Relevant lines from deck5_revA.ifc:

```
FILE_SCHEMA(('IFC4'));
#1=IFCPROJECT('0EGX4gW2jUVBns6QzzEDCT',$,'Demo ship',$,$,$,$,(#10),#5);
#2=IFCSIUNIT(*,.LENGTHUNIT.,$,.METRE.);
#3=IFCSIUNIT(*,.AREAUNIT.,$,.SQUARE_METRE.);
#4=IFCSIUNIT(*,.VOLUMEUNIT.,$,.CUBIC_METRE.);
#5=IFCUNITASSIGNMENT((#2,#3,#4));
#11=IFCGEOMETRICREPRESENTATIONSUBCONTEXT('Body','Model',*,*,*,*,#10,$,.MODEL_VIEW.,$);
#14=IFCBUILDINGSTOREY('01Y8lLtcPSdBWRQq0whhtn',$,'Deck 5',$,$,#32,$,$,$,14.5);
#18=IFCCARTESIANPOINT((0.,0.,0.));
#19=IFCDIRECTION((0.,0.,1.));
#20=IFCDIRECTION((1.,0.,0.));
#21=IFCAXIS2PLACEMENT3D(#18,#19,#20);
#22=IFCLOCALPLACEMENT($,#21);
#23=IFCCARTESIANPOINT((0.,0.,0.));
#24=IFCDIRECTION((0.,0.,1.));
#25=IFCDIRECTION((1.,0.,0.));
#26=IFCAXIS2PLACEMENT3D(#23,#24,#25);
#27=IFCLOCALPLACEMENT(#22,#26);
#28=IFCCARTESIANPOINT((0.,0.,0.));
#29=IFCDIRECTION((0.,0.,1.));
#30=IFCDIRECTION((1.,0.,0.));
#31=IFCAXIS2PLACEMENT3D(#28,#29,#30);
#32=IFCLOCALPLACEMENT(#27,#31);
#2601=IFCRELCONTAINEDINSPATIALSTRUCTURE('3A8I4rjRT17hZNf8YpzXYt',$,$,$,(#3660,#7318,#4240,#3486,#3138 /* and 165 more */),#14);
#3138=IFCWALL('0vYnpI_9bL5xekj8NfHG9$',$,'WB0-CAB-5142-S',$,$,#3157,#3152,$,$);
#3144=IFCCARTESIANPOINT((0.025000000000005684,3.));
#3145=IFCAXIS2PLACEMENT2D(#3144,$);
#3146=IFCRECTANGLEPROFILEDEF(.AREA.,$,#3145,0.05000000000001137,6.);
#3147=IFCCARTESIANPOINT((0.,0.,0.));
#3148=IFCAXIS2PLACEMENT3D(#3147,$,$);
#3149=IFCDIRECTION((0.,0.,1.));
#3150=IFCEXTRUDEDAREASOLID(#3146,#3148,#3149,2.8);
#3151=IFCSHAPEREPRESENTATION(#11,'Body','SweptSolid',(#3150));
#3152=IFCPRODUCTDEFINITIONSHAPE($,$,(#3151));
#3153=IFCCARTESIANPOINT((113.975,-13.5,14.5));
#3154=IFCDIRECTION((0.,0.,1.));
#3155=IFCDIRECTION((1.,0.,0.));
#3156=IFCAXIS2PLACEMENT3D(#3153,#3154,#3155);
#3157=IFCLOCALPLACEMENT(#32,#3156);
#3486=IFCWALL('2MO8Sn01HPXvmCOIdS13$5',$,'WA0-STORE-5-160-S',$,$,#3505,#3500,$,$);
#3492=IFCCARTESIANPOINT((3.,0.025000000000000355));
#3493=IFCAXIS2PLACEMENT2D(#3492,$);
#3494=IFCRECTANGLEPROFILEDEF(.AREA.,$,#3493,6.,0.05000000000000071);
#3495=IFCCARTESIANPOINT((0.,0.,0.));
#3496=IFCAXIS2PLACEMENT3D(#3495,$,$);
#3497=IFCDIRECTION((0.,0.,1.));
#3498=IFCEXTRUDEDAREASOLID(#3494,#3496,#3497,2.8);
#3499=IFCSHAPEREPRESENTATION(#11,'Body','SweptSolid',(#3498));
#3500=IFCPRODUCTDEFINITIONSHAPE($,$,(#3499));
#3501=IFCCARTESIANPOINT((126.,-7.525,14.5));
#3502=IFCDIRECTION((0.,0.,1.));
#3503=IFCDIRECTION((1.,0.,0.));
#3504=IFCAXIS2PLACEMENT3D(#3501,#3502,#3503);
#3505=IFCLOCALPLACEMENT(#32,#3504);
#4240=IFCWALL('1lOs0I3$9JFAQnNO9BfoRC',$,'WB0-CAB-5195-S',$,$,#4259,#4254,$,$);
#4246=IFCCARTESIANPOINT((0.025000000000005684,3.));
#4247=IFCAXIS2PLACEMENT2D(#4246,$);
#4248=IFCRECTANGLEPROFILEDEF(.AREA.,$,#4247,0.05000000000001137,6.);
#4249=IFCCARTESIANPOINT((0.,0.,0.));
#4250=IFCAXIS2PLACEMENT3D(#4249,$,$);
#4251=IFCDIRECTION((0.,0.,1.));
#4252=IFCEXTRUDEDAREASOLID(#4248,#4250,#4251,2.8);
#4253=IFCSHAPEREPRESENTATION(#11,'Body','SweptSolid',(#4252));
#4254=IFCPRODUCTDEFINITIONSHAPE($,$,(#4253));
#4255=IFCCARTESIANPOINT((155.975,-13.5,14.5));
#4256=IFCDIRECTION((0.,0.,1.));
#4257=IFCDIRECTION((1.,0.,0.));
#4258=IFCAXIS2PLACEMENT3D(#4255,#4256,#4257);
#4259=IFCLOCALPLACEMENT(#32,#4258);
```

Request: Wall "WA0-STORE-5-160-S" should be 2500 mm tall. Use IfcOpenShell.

```python
import ifcopenshell
import ifcopenshell.geom
import ifcopenshell.util.representation
import ifcopenshell.util.shape
import ifcopenshell.util.unit

model = ifcopenshell.open("deck5_revA.ifc")
unit_scale = ifcopenshell.util.unit.calculate_unit_scale(model)
settings = ifcopenshell.geom.settings()


def volume(element):
    """Net volume in cubic metres, openings subtracted."""
    shape = ifcopenshell.geom.create_shape(settings, element)
    return ifcopenshell.util.shape.get_volume(shape.geometry)


wall = model.by_guid("2MO8Sn01HPXvmCOIdS13$5")
before = volume(wall)

body = ifcopenshell.util.representation.get_representation(wall, "Model", "Body")
solid = body.Items[0]
old_height = solid.Depth
solid.Depth = 2.5 / unit_scale
after = volume(wall)

print(f"height {old_height:g} -> {solid.Depth:g}, volume {before:.3f} -> {after:.3f} m3")

model.write("deck5_revA-out.ifc")
```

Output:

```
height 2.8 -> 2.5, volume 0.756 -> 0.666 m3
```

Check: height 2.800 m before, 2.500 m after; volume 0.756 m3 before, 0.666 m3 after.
